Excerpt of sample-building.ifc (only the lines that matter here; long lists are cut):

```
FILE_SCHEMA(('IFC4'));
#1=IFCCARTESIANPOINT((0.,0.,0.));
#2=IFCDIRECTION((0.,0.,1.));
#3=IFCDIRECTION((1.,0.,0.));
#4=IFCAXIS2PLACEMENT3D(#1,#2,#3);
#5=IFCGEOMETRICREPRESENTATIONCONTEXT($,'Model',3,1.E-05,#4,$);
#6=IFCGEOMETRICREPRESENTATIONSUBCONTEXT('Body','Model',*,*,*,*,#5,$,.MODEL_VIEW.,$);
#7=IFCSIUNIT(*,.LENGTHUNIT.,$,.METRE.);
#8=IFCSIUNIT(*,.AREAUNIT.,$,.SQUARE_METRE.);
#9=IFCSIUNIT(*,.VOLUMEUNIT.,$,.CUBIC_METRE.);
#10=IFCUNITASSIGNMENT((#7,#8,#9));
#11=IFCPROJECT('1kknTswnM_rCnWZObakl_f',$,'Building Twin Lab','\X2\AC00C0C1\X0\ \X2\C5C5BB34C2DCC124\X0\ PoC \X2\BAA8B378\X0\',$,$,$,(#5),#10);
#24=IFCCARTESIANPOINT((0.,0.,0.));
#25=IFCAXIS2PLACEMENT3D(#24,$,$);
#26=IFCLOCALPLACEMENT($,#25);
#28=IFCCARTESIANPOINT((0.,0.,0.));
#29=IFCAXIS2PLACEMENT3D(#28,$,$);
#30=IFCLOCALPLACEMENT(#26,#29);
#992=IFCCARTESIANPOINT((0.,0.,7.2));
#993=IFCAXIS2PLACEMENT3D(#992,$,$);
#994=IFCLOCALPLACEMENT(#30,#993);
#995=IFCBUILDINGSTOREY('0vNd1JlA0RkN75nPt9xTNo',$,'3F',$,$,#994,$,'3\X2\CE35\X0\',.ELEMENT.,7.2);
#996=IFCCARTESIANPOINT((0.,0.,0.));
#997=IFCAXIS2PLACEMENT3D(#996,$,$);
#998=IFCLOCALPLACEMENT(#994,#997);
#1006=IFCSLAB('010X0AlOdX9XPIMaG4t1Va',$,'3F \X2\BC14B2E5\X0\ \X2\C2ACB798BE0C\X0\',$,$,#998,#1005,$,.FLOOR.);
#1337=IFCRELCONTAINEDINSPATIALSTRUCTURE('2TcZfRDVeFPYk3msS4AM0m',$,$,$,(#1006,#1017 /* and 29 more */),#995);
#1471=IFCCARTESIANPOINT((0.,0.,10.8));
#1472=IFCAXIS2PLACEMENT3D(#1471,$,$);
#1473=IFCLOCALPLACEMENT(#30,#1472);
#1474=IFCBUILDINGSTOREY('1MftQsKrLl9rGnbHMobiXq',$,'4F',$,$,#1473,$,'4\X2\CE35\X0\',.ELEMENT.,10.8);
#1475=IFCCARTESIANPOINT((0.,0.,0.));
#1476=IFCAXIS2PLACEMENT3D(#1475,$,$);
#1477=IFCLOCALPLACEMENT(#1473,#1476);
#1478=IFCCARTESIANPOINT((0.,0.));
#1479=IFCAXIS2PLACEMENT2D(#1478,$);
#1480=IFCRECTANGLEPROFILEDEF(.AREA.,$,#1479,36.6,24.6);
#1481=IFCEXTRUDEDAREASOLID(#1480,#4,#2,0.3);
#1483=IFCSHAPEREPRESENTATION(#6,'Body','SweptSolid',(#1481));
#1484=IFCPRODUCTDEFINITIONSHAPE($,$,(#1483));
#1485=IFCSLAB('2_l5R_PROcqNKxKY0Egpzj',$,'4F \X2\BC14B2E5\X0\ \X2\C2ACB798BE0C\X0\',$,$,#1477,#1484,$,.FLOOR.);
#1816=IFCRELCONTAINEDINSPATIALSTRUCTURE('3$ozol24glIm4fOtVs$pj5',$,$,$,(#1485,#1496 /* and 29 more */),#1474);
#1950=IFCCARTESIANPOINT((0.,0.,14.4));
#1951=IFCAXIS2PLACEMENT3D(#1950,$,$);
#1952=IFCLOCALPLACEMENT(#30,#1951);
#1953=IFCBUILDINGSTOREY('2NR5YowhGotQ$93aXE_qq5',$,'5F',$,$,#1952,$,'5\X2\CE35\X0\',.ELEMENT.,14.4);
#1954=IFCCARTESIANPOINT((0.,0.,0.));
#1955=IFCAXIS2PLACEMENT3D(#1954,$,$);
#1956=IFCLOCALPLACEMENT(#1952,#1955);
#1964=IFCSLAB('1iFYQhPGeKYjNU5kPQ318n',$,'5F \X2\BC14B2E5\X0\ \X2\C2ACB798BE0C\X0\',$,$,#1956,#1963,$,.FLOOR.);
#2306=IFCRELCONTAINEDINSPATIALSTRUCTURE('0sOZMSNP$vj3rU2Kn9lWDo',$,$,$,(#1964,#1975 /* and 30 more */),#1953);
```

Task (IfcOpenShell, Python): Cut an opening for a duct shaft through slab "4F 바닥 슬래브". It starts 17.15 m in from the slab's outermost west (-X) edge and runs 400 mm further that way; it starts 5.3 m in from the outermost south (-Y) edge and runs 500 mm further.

```python
import numpy as np
import ifcopenshell
import ifcopenshell.api.feature
import ifcopenshell.api.geometry
import ifcopenshell.api.root
import ifcopenshell.geom
import ifcopenshell.util.placement
import ifcopenshell.util.representation
import ifcopenshell.util.shape
import ifcopenshell.util.unit

model = ifcopenshell.open("sample-building.ifc")
unit_scale = ifcopenshell.util.unit.calculate_unit_scale(model)
settings = ifcopenshell.geom.settings()


def volume(element):
    """Net volume in cubic metres, openings subtracted."""
    shape = ifcopenshell.geom.create_shape(settings, element)
    return ifcopenshell.util.shape.get_volume(shape.geometry)


slab = model.by_guid("2_l5R_PROcqNKxKY0Egpzj")
before = volume(slab)

# Extent in the slab's own axes, in metres. The edges named are its -X and -Y sides.
slab_shape = ifcopenshell.geom.create_shape(settings, slab)
vertices = ifcopenshell.util.shape.get_vertices(slab_shape.geometry)
x_min, y_min, bottom = vertices.min(axis=0)
top = vertices[:, 2].max()

opening = ifcopenshell.api.root.create_entity(model, ifc_class="IfcOpeningElement", name="Duct shaft opening", predefined_type="OPENING")
context = ifcopenshell.util.representation.get_context(model, "Model", "Body", "MODEL_VIEW")
width, depth = 0.4, 0.5
outline = [(0.0, 0.0), (width, 0.0), (width, depth), (0.0, depth), (0.0, 0.0)]
# Overshoot both faces by 50 mm so the cut is clean.
shape = ifcopenshell.api.geometry.add_slab_representation(
    model, context=context, depth=top - bottom + 0.1, polyline=outline
)
ifcopenshell.api.geometry.assign_representation(model, product=opening, representation=shape)

matrix = ifcopenshell.util.placement.get_local_placement(slab.ObjectPlacement)
matrix[:, 3] = matrix @ np.append(np.array([x_min + 17.15, y_min + 5.3, bottom - 0.05]) / unit_scale, 1.0)
ifcopenshell.api.geometry.edit_object_placement(model, product=opening, matrix=matrix, is_si=False)
ifcopenshell.api.feature.add_feature(model, feature=opening, element=slab)

after = volume(slab)

print(f"slab volume {before:.3f} -> {after:.3f} m3")

model.write("sample-building_rev.ifc")
```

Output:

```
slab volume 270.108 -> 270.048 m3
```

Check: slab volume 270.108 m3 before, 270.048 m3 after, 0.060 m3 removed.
